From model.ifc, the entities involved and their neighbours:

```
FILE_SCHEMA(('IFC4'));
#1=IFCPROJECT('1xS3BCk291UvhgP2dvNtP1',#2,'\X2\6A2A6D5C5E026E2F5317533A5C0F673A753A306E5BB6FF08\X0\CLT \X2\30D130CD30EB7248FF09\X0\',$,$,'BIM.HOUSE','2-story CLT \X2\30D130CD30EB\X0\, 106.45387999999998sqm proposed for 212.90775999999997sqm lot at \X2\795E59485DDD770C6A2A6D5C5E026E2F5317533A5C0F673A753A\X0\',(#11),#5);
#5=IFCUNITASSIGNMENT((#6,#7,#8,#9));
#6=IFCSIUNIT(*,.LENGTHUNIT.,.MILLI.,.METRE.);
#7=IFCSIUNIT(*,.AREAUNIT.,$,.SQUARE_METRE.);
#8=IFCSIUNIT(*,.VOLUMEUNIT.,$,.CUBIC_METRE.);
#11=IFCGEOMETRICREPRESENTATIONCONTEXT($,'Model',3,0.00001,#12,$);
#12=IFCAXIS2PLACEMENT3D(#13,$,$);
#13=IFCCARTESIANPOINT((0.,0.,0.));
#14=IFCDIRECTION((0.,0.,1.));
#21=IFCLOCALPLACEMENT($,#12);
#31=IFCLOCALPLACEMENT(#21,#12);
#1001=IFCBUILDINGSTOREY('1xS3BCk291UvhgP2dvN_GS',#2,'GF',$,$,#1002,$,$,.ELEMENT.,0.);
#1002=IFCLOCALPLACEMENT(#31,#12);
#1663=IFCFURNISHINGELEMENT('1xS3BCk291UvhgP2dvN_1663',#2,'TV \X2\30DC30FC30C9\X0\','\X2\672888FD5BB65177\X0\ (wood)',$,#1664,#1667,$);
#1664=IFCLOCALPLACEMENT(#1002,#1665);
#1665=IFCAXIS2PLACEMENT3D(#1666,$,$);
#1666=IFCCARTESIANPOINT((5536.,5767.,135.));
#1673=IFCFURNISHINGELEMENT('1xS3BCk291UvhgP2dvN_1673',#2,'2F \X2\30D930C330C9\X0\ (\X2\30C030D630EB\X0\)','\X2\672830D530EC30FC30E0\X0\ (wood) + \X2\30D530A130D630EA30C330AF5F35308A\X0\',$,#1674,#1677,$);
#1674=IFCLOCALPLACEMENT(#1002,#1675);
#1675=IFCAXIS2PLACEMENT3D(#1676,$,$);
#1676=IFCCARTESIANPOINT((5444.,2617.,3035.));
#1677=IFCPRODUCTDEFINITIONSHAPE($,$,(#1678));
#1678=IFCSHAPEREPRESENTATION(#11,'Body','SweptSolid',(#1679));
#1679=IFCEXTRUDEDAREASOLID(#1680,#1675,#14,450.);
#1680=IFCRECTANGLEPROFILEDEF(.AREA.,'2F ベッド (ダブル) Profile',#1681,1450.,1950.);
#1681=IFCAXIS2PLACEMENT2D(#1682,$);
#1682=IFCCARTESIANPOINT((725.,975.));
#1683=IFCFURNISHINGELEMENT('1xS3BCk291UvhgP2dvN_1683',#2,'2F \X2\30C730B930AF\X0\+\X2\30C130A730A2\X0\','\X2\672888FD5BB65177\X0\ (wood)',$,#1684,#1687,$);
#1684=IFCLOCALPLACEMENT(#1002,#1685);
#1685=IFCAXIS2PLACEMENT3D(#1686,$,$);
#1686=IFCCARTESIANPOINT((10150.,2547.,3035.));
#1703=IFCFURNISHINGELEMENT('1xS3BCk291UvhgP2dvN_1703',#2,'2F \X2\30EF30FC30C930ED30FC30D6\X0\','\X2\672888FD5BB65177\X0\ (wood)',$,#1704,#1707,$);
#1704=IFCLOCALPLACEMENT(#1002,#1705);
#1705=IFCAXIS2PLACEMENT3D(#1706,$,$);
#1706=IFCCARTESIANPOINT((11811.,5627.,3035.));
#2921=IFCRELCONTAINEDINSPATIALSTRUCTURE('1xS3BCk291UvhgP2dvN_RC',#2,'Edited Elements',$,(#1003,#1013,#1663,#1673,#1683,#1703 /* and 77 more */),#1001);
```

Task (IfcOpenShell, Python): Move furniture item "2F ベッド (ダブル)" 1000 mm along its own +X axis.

```python
import ifcopenshell
import ifcopenshell.api.geometry
import ifcopenshell.util.placement
import ifcopenshell.util.unit

model = ifcopenshell.open("model.ifc")
unit_scale = ifcopenshell.util.unit.calculate_unit_scale(model)

item = model.by_guid("1xS3BCk291UvhgP2dvN_1673")
matrix = ifcopenshell.util.placement.get_local_placement(item.ObjectPlacement)
matrix[:3, 3] += matrix[:3, 0] * 1 / unit_scale
ifcopenshell.api.geometry.edit_object_placement(model, product=item, matrix=matrix, is_si=False)

print(ifcopenshell.util.placement.get_local_placement(item.ObjectPlacement).round(3) + 0.0)

model.write("model_v2.ifc")
```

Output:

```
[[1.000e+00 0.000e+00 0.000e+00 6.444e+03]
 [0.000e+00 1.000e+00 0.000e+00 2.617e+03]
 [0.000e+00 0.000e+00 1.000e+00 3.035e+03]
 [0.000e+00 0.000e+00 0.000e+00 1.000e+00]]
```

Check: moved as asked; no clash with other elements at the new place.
